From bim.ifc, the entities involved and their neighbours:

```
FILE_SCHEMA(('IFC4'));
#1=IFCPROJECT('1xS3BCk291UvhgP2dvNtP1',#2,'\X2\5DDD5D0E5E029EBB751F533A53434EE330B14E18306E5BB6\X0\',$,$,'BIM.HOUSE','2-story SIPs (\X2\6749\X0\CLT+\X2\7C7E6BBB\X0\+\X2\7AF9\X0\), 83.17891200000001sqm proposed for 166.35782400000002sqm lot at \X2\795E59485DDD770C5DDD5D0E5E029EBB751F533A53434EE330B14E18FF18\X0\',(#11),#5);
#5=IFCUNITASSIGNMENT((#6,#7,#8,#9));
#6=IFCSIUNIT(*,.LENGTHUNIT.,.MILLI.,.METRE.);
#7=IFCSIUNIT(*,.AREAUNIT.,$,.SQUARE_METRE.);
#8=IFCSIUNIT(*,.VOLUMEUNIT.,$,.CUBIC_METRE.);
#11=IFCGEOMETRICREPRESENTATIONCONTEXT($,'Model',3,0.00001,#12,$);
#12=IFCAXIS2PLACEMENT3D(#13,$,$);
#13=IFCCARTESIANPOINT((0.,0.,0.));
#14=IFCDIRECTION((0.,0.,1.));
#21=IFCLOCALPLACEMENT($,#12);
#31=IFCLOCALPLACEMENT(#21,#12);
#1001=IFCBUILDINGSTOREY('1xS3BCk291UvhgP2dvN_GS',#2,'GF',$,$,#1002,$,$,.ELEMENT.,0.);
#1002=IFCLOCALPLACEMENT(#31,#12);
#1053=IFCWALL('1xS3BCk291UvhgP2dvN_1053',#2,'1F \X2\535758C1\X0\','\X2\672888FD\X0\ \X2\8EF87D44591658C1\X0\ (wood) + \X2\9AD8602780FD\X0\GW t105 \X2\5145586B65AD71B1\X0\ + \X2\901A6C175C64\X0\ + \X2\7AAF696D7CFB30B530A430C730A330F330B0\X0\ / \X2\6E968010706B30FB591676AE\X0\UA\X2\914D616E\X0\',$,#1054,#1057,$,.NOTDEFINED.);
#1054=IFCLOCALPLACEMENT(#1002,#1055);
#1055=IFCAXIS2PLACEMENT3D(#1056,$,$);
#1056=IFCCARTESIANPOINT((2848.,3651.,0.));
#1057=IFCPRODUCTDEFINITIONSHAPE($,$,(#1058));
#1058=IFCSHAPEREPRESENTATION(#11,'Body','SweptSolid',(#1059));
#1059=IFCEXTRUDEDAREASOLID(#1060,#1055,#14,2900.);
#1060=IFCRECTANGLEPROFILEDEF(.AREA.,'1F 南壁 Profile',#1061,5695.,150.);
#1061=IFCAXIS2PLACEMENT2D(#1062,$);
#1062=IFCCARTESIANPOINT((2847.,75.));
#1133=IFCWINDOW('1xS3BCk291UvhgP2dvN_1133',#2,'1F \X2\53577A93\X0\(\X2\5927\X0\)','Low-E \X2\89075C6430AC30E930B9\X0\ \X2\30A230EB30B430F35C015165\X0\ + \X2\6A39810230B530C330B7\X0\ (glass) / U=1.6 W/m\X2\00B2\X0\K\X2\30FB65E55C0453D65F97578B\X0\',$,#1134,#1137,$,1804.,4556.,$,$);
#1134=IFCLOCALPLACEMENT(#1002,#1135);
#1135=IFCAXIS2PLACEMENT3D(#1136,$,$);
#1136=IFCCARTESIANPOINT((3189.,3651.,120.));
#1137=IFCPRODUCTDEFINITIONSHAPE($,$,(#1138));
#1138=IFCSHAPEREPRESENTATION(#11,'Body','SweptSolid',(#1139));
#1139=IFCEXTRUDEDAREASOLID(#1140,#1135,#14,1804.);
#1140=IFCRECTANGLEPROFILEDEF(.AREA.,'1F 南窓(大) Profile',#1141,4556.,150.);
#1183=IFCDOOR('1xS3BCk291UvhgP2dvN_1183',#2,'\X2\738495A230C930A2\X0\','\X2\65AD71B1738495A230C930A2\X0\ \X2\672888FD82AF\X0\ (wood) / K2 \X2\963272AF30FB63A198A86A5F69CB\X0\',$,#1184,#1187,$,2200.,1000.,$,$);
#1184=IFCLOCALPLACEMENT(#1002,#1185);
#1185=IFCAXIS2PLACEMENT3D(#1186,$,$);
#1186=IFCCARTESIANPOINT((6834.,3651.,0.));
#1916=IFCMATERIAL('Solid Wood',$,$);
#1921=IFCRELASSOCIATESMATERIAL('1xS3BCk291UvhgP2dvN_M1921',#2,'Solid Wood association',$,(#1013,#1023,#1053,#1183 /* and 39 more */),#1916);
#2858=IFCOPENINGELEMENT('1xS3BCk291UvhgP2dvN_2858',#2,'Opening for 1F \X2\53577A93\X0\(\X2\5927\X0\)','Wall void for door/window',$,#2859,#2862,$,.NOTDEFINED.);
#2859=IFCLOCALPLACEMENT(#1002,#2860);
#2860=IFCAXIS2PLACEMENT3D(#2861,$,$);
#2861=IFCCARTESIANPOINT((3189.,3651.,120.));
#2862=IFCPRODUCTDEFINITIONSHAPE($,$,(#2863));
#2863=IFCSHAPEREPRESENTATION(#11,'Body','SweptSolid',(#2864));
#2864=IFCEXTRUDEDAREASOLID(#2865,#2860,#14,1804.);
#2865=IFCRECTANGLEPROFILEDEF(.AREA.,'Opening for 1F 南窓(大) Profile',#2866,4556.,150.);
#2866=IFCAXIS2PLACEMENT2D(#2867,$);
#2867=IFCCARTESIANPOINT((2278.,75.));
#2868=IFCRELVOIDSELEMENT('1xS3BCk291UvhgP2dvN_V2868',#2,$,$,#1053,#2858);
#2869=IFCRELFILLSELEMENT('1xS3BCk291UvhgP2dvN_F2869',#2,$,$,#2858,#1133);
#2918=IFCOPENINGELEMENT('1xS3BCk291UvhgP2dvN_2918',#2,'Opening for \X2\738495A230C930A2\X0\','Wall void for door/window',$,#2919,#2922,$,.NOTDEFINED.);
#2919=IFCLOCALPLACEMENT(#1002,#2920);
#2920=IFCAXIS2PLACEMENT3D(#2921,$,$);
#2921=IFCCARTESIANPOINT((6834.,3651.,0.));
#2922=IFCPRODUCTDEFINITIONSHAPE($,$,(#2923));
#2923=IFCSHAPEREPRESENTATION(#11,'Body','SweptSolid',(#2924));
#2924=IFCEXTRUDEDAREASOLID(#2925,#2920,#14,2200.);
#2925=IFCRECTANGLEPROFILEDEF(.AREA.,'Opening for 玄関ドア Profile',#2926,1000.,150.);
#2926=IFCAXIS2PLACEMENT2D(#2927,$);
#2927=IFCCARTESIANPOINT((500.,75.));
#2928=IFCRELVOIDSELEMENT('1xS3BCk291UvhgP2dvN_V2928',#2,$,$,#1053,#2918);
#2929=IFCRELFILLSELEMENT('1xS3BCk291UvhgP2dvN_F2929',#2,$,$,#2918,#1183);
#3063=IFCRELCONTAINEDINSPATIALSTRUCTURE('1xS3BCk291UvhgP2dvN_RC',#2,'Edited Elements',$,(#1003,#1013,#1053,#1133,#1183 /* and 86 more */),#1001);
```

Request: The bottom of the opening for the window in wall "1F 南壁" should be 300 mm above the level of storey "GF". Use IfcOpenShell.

```python
import numpy as np
import ifcopenshell
import ifcopenshell.api.geometry
import ifcopenshell.geom
import ifcopenshell.util.element
import ifcopenshell.util.placement
import ifcopenshell.util.shape
import ifcopenshell.util.unit

model = ifcopenshell.open("bim.ifc")
unit_scale = ifcopenshell.util.unit.calculate_unit_scale(model)

window = model.by_guid("1xS3BCk291UvhgP2dvN_1133")
opening = window.FillsVoids[0].RelatingOpeningElement
storey = ifcopenshell.util.element.get_container(window, ifc_class="IfcBuildingStorey")
level = ifcopenshell.util.placement.get_local_placement(storey.ObjectPlacement)[2, 3]

# The opening's origin need not be at the sill, so measure its lowest point.
shape = ifcopenshell.geom.create_shape(ifcopenshell.geom.settings(), opening)
bottom = ifcopenshell.util.shape.get_shape_bottom_elevation(shape, shape.geometry) / unit_scale
dz = level + 0.3 / unit_scale - bottom

shift = np.array([0.0, 0.0, dz])
# The window is not placed relative to its opening, so move both.
for product in (opening, window):
    matrix = ifcopenshell.util.placement.get_local_placement(product.ObjectPlacement)
    matrix[:3, 3] += shift
    ifcopenshell.api.geometry.edit_object_placement(model, product=product, matrix=matrix, is_si=False)

print(f"moved by {dz * unit_scale:+.3f} m")

model.write("bim_edited.ifc")
```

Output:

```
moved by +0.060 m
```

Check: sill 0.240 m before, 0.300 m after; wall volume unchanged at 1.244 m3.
